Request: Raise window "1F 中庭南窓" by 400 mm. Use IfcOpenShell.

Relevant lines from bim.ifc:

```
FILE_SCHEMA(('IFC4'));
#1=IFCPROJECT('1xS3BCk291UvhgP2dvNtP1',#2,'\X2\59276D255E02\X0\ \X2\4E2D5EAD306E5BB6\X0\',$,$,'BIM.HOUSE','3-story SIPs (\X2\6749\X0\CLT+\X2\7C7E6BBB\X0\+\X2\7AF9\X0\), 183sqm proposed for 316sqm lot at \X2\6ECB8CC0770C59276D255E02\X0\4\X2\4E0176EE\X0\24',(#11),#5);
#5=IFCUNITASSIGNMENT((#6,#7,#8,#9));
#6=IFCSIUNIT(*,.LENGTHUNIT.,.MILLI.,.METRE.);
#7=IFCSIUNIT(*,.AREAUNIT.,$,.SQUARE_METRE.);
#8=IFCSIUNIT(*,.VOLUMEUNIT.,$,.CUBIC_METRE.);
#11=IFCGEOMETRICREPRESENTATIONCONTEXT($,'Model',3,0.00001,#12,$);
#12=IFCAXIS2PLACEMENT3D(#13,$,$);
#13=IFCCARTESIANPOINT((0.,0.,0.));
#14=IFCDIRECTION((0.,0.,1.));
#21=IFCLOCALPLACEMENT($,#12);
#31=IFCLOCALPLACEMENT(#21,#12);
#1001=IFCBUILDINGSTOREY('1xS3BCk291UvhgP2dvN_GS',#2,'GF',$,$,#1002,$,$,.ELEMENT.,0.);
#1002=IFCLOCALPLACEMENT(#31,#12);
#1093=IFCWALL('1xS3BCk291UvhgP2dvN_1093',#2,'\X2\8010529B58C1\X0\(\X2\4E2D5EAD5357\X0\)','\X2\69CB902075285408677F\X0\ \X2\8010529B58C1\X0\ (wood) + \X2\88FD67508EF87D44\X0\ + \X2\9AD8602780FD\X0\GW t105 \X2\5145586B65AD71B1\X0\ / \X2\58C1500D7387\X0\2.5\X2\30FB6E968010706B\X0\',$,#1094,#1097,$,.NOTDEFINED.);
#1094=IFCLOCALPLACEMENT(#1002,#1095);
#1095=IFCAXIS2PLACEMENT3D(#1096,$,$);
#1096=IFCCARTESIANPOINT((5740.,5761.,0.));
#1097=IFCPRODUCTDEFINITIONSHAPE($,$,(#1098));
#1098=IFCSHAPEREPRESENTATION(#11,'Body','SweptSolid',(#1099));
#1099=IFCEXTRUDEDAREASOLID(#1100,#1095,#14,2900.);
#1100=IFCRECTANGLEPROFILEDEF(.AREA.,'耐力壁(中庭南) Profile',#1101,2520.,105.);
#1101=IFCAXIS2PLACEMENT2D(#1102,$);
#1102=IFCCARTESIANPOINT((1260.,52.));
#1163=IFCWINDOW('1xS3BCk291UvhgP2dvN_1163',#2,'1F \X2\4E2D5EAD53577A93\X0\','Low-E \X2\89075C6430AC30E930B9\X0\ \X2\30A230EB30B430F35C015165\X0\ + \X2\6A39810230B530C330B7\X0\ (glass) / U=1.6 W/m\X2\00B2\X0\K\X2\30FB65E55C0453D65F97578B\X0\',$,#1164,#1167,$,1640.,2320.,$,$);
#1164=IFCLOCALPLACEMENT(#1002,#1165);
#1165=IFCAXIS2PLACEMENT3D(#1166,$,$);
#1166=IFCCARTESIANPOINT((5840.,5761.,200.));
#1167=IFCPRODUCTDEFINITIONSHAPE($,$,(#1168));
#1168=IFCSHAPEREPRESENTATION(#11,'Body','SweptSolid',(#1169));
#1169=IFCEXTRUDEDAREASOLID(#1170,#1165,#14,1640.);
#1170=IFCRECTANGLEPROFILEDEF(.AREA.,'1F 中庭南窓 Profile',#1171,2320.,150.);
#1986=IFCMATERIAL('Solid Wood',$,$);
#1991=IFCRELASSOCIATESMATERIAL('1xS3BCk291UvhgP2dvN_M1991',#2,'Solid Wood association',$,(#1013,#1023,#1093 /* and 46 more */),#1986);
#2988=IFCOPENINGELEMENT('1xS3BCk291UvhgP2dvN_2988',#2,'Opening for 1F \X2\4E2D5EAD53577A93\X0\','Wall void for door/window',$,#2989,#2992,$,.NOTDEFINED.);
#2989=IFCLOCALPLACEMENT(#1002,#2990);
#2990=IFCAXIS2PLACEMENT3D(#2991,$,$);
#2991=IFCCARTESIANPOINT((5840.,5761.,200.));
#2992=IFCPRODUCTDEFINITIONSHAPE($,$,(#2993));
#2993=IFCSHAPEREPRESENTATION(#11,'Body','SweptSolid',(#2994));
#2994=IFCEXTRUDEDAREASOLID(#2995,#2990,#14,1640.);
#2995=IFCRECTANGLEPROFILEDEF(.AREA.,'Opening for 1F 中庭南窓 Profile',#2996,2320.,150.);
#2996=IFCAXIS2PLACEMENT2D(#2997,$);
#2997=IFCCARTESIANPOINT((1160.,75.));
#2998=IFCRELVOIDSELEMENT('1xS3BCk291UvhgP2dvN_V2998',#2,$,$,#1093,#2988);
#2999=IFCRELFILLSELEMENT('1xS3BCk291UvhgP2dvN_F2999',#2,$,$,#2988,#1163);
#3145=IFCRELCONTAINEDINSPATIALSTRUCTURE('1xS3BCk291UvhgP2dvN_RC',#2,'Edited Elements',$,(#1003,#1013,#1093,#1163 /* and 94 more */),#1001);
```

```python
import numpy as np
import ifcopenshell
import ifcopenshell.api.geometry
import ifcopenshell.util.placement
import ifcopenshell.util.unit

model = ifcopenshell.open("bim.ifc")
unit_scale = ifcopenshell.util.unit.calculate_unit_scale(model)

window = model.by_guid("1xS3BCk291UvhgP2dvN_1163")
opening = window.FillsVoids[0].RelatingOpeningElement
dz = 0.4 / unit_scale

shift = np.array([0.0, 0.0, dz])
# The window is not placed relative to its opening, so move both.
for product in (opening, window):
    matrix = ifcopenshell.util.placement.get_local_placement(product.ObjectPlacement)
    matrix[:3, 3] += shift
    ifcopenshell.api.geometry.edit_object_placement(model, product=product, matrix=matrix, is_si=False)

print(f"moved by {dz * unit_scale:+.3f} m")

model.write("bim_updated.ifc")
```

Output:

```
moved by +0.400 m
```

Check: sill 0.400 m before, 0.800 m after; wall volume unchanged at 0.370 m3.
